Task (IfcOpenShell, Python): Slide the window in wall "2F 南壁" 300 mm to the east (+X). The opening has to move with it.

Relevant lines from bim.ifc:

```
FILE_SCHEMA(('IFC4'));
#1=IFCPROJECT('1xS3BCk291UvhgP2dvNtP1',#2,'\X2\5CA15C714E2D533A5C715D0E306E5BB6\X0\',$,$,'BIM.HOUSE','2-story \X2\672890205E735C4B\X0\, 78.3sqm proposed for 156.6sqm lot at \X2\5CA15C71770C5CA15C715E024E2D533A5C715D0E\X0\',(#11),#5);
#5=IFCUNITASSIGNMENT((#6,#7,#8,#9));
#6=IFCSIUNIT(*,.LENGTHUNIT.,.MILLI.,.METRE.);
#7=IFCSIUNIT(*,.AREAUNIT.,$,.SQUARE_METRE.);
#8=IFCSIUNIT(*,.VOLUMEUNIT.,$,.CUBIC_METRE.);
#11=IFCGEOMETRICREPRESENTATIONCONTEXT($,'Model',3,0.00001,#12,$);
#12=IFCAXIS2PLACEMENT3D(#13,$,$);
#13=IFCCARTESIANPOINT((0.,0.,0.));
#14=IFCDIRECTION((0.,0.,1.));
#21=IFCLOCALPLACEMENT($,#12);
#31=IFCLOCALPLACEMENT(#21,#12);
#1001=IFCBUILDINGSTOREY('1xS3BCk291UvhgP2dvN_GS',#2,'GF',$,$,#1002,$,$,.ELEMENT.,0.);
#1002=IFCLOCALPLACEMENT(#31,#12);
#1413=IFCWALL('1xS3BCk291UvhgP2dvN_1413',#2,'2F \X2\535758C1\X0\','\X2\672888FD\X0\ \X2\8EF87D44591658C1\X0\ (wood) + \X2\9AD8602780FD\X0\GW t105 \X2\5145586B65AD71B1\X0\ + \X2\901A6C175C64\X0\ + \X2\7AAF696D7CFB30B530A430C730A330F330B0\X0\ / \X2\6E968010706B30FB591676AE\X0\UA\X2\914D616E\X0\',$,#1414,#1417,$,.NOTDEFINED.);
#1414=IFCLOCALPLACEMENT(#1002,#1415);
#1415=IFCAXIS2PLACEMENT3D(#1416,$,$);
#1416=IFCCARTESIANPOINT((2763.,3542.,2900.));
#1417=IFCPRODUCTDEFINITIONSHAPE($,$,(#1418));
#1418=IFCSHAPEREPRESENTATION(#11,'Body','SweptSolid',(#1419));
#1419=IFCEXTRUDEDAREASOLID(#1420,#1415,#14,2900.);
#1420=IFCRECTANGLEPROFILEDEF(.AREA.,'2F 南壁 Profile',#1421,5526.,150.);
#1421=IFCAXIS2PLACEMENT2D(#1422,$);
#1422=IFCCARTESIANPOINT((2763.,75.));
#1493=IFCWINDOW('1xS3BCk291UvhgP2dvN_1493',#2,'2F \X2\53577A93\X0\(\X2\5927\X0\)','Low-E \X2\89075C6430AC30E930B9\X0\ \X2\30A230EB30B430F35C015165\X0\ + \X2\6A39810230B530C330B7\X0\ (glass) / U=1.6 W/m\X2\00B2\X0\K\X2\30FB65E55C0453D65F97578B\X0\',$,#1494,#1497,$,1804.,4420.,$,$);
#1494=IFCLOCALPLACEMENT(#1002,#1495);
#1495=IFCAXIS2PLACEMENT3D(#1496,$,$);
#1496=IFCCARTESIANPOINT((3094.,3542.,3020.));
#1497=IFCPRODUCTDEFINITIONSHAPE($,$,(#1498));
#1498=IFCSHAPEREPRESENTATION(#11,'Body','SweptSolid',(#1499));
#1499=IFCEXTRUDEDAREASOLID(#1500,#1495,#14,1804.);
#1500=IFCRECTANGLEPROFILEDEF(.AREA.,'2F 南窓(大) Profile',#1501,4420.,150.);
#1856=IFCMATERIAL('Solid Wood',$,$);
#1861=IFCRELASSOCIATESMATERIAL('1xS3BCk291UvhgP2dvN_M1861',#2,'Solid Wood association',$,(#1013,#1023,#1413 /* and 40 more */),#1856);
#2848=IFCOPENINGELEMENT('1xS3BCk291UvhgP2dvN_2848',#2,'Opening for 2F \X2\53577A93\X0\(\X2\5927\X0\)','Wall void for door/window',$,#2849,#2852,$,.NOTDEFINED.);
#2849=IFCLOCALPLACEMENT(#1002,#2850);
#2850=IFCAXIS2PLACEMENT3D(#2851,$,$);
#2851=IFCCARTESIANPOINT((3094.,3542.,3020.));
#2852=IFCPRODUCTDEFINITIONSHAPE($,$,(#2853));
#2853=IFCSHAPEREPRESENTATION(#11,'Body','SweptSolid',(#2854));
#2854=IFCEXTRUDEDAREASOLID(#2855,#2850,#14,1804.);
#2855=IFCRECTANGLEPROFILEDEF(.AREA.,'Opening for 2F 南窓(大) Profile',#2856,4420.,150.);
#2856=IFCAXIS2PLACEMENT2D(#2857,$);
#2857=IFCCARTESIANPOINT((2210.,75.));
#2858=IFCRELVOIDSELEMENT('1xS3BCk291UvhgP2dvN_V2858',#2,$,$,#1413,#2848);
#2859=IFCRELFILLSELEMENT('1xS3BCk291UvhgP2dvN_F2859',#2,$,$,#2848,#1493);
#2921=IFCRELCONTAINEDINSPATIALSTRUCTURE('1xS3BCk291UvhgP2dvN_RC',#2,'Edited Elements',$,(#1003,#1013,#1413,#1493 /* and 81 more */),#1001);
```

```python
import ifcopenshell
import ifcopenshell.api.geometry
import ifcopenshell.util.placement

model = ifcopenshell.open("bim.ifc")

window = model.by_guid("1xS3BCk291UvhgP2dvN_1493")
opening = window.FillsVoids[0].RelatingOpeningElement
wall = opening.VoidsElements[0].RelatingBuildingElement

wall_matrix = ifcopenshell.util.placement.get_local_placement(wall.ObjectPlacement)
shift = wall_matrix[:3, 0] * 300.0
before = ifcopenshell.util.placement.get_local_placement(window.ObjectPlacement)[:3, 3].copy()

# The window is not placed relative to its opening, so move both.
for product in (opening, window):
    matrix = ifcopenshell.util.placement.get_local_placement(product.ObjectPlacement)
    matrix[:3, 3] += shift
    ifcopenshell.api.geometry.edit_object_placement(model, product=product, matrix=matrix, is_si=False)

after = ifcopenshell.util.placement.get_local_placement(window.ObjectPlacement)[:3, 3]
print("window moved by", (after - before).round(3) + 0.0)

model.write("bim_updated.ifc")
```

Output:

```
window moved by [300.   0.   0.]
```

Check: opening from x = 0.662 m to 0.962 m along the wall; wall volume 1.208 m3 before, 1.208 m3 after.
